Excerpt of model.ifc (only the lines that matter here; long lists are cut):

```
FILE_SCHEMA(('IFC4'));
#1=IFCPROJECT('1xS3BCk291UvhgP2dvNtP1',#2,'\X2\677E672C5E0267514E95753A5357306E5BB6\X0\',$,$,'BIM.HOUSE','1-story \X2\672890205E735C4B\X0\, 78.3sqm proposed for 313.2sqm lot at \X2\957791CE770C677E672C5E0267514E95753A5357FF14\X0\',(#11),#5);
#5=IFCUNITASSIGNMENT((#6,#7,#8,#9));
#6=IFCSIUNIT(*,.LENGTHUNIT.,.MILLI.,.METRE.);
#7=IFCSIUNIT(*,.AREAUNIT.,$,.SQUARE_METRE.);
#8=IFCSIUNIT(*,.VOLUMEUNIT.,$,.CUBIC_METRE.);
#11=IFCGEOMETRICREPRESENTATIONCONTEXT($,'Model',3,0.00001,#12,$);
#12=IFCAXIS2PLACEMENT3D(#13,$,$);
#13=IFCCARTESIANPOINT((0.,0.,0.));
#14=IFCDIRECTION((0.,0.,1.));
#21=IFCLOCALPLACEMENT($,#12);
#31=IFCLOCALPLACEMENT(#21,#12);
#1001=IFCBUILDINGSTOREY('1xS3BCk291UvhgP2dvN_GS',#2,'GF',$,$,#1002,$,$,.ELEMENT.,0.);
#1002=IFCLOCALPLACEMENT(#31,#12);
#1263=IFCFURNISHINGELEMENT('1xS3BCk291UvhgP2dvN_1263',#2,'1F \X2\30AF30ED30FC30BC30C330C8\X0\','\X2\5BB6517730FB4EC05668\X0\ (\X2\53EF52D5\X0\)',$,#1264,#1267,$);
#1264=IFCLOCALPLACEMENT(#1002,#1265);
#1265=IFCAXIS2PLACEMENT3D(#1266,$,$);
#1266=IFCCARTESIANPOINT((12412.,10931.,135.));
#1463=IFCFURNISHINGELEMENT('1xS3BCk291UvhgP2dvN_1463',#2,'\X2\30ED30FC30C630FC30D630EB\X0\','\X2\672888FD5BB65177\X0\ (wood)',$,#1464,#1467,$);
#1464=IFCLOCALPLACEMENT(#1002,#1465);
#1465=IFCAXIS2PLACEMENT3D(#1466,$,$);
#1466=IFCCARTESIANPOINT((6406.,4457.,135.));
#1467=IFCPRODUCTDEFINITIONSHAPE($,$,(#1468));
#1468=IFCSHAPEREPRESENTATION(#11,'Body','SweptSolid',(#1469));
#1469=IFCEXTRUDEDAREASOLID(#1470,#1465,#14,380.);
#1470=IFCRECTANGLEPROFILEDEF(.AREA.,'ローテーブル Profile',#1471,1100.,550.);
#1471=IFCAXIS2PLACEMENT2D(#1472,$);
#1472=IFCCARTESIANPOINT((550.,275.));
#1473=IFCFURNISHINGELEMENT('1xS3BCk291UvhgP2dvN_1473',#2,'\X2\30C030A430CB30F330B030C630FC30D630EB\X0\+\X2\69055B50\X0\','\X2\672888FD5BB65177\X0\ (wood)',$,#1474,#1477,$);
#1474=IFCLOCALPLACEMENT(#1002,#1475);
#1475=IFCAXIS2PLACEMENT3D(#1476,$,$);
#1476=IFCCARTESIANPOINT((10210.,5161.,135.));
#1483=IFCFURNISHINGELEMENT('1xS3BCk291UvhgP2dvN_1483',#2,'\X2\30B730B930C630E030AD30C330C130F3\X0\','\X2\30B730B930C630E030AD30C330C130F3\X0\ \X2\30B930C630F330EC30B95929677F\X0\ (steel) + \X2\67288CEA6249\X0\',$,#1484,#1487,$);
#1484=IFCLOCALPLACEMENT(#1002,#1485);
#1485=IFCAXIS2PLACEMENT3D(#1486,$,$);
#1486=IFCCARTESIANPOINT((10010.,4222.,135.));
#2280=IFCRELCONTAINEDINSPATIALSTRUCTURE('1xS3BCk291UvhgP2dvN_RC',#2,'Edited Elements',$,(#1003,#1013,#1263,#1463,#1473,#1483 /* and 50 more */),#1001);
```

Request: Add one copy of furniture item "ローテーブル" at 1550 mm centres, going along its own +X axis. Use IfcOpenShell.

```python
import ifcopenshell
import ifcopenshell.api.geometry
import ifcopenshell.api.root
import ifcopenshell.util.element
import ifcopenshell.util.placement

model = ifcopenshell.open("model.ifc")


def reuse_history(source, copy):
    """copy_class also copies each property set's owner history, people and application; keep the originals."""
    for rel in copy.IsDefinedBy:
        if rel.is_a("IfcRelDefinesByProperties") and (history := rel.RelatingPropertyDefinition.OwnerHistory):
            rel.RelatingPropertyDefinition.OwnerHistory = source.OwnerHistory
            ifcopenshell.util.element.remove_deep2(model, history)


source = model.by_guid("1xS3BCk291UvhgP2dvN_1463")
base = ifcopenshell.util.placement.get_local_placement(source.ObjectPlacement)
step = base[:3, 0] * 1550.0

for i in range(1, 2):
    copy = ifcopenshell.api.root.copy_class(model, product=source)
    copy.Representation = ifcopenshell.util.element.copy_deep(
        model, source.Representation, exclude=["IfcGeometricRepresentationContext", "IfcRepresentationMap"]
    )
    reuse_history(source, copy)
    matrix = base.copy()
    matrix[:3, 3] += i * step
    print("added at", matrix[:3, 3].round(3) + 0.0)
    ifcopenshell.api.geometry.edit_object_placement(model, product=copy, matrix=matrix, is_si=False)

model.write("model_v2.ifc")
```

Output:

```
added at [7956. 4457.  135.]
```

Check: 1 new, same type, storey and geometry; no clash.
